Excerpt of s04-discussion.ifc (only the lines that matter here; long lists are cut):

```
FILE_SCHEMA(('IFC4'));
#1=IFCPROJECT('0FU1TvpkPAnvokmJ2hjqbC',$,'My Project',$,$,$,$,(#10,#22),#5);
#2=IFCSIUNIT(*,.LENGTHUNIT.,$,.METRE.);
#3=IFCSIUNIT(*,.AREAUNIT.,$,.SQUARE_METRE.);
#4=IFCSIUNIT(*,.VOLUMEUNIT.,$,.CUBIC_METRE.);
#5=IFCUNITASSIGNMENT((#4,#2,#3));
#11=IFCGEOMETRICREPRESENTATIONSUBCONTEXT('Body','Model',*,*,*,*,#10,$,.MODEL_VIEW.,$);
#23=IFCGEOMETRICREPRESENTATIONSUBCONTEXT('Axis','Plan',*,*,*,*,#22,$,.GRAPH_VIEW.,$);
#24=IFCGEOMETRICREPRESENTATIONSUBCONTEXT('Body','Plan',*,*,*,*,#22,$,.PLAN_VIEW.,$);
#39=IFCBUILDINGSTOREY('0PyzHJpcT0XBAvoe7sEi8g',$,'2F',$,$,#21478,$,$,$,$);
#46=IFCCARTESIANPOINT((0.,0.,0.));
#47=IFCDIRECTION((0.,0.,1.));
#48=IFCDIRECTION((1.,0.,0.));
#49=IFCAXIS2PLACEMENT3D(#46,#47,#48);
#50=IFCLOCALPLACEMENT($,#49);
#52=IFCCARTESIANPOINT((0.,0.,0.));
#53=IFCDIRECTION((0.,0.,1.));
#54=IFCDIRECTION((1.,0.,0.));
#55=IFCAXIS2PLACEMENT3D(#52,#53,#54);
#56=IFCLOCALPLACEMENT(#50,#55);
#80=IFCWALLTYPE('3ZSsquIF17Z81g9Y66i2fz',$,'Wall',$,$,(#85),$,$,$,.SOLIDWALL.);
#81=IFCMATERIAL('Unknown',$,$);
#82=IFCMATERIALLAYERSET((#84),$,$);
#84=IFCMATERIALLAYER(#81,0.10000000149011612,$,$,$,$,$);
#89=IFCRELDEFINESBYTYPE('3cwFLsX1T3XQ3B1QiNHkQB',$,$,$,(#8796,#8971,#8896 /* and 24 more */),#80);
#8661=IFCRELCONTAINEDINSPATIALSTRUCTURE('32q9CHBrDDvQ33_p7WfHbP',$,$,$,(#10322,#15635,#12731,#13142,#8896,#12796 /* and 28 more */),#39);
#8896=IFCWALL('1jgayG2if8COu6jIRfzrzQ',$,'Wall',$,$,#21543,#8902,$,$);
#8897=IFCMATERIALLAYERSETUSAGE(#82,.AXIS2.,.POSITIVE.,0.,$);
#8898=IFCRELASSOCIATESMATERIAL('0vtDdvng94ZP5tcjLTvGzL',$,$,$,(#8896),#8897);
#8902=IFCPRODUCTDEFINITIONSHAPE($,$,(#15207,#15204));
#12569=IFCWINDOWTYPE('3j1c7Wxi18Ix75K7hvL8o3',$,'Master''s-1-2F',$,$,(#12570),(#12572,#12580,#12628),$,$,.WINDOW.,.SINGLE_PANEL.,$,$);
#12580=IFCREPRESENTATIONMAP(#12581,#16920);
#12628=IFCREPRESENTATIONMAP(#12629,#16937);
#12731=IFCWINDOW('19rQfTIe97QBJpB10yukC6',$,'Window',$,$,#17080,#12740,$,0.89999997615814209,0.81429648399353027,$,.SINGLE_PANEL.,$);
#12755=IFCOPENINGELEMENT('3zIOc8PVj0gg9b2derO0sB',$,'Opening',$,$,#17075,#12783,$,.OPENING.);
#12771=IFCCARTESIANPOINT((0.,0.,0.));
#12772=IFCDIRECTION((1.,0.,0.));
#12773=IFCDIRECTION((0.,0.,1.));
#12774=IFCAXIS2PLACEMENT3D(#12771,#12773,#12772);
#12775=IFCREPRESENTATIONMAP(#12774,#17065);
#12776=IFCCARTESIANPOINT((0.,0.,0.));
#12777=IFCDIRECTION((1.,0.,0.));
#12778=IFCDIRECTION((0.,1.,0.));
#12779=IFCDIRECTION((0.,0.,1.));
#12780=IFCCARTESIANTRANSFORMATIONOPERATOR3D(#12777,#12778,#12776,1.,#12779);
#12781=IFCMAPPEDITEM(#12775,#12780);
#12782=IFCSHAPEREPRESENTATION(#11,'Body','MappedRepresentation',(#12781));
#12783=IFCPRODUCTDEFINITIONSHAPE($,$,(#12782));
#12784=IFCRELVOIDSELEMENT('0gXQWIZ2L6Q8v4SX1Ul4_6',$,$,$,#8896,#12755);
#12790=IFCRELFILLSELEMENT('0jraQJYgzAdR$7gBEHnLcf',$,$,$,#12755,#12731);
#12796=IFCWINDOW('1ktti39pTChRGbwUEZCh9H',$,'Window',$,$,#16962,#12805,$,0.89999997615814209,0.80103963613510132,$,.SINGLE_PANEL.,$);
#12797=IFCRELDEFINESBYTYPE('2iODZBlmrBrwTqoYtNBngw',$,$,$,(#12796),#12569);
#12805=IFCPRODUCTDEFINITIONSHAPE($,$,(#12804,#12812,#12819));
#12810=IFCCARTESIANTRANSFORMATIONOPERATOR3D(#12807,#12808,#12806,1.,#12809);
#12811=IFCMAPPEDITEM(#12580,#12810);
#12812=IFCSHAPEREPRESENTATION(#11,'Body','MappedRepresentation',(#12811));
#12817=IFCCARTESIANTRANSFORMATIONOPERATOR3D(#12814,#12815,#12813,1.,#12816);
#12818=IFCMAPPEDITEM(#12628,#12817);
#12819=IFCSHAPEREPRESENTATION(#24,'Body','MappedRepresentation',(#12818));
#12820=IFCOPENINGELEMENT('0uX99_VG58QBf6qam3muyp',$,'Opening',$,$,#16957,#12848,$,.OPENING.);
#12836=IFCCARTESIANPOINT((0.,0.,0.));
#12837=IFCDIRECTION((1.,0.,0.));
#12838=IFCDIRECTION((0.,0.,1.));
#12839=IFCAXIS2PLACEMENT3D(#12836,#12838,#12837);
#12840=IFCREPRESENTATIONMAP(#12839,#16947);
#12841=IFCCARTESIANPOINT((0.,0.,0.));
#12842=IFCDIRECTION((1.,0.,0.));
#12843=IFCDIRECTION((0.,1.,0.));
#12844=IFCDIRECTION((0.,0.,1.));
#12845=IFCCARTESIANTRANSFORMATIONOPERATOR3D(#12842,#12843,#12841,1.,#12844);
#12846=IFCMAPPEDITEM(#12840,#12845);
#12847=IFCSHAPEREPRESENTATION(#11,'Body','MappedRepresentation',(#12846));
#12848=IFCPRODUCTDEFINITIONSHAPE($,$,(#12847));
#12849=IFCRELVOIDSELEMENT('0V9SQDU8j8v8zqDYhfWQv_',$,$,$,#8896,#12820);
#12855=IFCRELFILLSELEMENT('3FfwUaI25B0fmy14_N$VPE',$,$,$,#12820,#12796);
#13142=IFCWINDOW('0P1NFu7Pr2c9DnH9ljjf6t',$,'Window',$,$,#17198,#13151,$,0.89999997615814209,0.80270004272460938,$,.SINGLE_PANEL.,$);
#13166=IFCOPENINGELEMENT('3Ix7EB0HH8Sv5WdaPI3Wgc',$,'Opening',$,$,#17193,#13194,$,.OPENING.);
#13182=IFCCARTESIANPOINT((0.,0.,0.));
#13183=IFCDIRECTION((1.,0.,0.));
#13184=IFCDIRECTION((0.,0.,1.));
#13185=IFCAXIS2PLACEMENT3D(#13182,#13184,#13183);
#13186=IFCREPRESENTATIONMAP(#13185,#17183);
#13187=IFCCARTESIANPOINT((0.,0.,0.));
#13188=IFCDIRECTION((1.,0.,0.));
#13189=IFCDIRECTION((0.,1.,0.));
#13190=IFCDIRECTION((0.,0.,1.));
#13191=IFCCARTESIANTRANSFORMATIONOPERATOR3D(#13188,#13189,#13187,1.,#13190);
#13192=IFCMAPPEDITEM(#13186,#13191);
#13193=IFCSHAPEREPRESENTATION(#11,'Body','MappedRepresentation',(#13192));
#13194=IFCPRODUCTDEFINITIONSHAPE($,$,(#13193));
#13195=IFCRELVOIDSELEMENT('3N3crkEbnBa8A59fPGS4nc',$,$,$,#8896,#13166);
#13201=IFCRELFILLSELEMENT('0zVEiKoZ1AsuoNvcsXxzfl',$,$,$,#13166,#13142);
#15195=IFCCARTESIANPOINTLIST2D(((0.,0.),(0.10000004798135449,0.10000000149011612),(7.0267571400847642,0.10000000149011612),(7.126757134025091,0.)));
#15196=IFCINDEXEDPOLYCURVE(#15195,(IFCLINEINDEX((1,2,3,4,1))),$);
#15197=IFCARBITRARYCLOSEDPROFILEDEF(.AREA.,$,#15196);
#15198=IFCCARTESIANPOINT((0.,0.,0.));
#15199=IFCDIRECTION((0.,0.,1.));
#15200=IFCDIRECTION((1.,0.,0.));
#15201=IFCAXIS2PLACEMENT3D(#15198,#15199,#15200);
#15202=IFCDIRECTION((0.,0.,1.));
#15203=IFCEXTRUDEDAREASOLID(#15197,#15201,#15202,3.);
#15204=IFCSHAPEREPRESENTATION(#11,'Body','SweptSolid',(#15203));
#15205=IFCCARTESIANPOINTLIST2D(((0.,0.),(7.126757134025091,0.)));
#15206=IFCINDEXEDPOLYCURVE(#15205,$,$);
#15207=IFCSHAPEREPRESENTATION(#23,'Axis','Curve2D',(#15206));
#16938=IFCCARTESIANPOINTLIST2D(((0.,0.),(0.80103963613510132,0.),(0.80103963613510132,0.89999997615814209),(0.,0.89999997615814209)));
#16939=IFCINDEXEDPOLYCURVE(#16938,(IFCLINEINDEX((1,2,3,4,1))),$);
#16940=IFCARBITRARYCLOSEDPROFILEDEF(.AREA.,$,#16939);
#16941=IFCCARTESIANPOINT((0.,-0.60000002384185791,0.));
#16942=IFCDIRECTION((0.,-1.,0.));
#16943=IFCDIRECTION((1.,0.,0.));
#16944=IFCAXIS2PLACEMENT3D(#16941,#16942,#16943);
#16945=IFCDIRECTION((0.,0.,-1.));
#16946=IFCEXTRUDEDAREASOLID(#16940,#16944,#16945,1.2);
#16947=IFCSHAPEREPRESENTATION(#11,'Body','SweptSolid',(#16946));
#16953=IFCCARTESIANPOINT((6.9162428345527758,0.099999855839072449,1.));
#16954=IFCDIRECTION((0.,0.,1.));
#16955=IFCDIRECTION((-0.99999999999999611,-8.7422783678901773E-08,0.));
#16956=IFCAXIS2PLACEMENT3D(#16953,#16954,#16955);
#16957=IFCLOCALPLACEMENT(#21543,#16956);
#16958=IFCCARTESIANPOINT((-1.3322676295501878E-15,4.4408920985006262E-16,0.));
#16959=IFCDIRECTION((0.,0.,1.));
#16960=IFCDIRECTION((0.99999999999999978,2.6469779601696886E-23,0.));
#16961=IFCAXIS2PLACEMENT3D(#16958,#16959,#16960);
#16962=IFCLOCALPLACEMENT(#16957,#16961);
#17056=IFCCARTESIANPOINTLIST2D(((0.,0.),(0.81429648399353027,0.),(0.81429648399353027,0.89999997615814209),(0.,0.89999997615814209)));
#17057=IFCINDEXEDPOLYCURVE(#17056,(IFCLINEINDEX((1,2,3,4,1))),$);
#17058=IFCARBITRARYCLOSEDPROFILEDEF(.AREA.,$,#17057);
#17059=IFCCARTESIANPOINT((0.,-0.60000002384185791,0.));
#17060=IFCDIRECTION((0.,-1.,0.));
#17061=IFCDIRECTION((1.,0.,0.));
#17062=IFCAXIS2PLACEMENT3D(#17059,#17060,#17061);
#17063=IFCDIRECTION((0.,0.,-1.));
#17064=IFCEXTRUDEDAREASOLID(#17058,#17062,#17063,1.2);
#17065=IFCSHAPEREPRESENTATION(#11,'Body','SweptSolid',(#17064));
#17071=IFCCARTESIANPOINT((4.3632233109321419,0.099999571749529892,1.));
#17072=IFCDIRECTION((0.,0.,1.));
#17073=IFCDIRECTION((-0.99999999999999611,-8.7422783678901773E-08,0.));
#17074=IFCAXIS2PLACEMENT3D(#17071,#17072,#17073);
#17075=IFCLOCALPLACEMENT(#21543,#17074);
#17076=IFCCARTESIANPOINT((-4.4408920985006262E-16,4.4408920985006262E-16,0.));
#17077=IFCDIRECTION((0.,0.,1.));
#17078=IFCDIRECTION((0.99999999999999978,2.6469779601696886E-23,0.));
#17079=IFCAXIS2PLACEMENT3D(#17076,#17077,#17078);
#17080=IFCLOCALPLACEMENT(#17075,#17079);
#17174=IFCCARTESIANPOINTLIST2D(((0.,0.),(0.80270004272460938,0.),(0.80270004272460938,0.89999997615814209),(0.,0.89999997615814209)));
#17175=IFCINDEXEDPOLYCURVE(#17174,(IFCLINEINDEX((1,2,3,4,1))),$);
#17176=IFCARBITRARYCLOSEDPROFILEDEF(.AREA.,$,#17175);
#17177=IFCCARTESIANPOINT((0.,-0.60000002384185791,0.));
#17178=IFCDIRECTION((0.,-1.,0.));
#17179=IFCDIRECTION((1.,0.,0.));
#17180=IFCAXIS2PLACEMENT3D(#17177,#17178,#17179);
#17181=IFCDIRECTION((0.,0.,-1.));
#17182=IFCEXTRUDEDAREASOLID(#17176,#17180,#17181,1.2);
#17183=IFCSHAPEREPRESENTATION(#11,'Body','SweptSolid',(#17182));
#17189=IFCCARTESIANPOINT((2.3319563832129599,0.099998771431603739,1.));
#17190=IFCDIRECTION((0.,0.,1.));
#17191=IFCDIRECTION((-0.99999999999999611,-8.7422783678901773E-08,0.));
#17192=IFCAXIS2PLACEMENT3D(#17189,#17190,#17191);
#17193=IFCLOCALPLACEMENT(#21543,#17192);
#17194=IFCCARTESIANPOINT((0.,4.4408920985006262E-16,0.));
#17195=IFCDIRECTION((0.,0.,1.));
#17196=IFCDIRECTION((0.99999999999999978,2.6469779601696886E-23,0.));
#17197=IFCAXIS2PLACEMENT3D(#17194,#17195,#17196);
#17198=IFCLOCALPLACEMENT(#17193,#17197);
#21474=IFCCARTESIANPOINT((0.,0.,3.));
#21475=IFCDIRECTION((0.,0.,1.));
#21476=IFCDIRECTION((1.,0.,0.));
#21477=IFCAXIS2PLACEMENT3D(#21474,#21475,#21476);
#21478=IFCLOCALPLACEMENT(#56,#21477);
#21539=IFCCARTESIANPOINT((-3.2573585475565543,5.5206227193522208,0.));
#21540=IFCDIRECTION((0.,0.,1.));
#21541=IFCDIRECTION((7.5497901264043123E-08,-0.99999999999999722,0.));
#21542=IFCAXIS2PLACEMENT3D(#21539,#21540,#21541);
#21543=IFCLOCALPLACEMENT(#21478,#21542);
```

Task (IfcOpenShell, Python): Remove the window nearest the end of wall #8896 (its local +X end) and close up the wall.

```python
import ifcopenshell
import ifcopenshell.api.feature
import ifcopenshell.api.root
import ifcopenshell.geom
import ifcopenshell.util.shape

model = ifcopenshell.open("s04-discussion.ifc")
settings = ifcopenshell.geom.settings()


def volume(element):
    """Net volume in cubic metres, openings subtracted."""
    shape = ifcopenshell.geom.create_shape(settings, element)
    return ifcopenshell.util.shape.get_volume(shape.geometry)


window = model.by_guid("1ktti39pTChRGbwUEZCh9H")
opening = window.FillsVoids[0].RelatingOpeningElement
wall = opening.VoidsElements[0].RelatingBuildingElement
before = volume(wall)

ifcopenshell.api.root.remove_product(model, product=window)
ifcopenshell.api.feature.remove_feature(model, feature=opening)

after = volume(wall)

print(f"wall volume {before:.3f} -> {after:.3f} m3")

model.write("s04-discussion_edited.ifc")
```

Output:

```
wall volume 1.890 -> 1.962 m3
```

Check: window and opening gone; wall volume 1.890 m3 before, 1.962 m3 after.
